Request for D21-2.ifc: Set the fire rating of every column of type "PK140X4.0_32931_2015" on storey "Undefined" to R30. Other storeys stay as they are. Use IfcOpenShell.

First a look at what the model holds.

```python
import ifcopenshell
import ifcopenshell.util.element

model = ifcopenshell.open("D21-2.ifc")
print(model.schema)
storey = next(s for s in model.by_type("IfcBuildingStorey") if s.Name == "Undefined")
columns = [e for e in ifcopenshell.util.element.get_decomposition(storey) if e.is_a("IfcColumn")]
seen = {}
for e in columns:
    element_type = ifcopenshell.util.element.get_type(e)
    key = (element_type.Name if element_type != e and element_type else None, ifcopenshell.util.element.get_pset(e, "Pset_ColumnCommon", "FireRating"))
    seen[key] = seen.get(key, 0) + 1
for (name, value), count in sorted(seen.items(), key=str):
    print(count, "x", name, "|", value)
```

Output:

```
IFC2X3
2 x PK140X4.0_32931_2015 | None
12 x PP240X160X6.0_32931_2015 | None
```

```python
import ifcopenshell
import ifcopenshell.api.pset
import ifcopenshell.util.element

model = ifcopenshell.open("D21-2.ifc")

storey = next(s for s in model.by_type("IfcBuildingStorey") if s.Name == "Undefined")
columns = [e for e in ifcopenshell.util.element.get_decomposition(storey) if e.is_a("IfcColumn")]

count = 0
for e in columns:
    element_type = ifcopenshell.util.element.get_type(e)
    if element_type in (None, e) or element_type.Name != "PK140X4.0_32931_2015":
        continue
    found = ifcopenshell.util.element.get_pset(e, "Pset_ColumnCommon", should_inherit=False)
    if found:
        pset = model.by_id(found["id"])
        if len(ifcopenshell.util.element.get_elements_by_pset(pset)) > 1:
            pset = ifcopenshell.api.pset.unshare_pset(model, products=[e], pset=pset)[0]
    else:
        pset = ifcopenshell.api.pset.add_pset(model, product=e, name="Pset_ColumnCommon")
    ifcopenshell.api.pset.edit_pset(model, pset=pset, properties={"FireRating": "R30"})
    count += 1

print(count, "columns updated")

model.write("D21-2_edited.ifc")
```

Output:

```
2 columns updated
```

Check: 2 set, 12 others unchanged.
